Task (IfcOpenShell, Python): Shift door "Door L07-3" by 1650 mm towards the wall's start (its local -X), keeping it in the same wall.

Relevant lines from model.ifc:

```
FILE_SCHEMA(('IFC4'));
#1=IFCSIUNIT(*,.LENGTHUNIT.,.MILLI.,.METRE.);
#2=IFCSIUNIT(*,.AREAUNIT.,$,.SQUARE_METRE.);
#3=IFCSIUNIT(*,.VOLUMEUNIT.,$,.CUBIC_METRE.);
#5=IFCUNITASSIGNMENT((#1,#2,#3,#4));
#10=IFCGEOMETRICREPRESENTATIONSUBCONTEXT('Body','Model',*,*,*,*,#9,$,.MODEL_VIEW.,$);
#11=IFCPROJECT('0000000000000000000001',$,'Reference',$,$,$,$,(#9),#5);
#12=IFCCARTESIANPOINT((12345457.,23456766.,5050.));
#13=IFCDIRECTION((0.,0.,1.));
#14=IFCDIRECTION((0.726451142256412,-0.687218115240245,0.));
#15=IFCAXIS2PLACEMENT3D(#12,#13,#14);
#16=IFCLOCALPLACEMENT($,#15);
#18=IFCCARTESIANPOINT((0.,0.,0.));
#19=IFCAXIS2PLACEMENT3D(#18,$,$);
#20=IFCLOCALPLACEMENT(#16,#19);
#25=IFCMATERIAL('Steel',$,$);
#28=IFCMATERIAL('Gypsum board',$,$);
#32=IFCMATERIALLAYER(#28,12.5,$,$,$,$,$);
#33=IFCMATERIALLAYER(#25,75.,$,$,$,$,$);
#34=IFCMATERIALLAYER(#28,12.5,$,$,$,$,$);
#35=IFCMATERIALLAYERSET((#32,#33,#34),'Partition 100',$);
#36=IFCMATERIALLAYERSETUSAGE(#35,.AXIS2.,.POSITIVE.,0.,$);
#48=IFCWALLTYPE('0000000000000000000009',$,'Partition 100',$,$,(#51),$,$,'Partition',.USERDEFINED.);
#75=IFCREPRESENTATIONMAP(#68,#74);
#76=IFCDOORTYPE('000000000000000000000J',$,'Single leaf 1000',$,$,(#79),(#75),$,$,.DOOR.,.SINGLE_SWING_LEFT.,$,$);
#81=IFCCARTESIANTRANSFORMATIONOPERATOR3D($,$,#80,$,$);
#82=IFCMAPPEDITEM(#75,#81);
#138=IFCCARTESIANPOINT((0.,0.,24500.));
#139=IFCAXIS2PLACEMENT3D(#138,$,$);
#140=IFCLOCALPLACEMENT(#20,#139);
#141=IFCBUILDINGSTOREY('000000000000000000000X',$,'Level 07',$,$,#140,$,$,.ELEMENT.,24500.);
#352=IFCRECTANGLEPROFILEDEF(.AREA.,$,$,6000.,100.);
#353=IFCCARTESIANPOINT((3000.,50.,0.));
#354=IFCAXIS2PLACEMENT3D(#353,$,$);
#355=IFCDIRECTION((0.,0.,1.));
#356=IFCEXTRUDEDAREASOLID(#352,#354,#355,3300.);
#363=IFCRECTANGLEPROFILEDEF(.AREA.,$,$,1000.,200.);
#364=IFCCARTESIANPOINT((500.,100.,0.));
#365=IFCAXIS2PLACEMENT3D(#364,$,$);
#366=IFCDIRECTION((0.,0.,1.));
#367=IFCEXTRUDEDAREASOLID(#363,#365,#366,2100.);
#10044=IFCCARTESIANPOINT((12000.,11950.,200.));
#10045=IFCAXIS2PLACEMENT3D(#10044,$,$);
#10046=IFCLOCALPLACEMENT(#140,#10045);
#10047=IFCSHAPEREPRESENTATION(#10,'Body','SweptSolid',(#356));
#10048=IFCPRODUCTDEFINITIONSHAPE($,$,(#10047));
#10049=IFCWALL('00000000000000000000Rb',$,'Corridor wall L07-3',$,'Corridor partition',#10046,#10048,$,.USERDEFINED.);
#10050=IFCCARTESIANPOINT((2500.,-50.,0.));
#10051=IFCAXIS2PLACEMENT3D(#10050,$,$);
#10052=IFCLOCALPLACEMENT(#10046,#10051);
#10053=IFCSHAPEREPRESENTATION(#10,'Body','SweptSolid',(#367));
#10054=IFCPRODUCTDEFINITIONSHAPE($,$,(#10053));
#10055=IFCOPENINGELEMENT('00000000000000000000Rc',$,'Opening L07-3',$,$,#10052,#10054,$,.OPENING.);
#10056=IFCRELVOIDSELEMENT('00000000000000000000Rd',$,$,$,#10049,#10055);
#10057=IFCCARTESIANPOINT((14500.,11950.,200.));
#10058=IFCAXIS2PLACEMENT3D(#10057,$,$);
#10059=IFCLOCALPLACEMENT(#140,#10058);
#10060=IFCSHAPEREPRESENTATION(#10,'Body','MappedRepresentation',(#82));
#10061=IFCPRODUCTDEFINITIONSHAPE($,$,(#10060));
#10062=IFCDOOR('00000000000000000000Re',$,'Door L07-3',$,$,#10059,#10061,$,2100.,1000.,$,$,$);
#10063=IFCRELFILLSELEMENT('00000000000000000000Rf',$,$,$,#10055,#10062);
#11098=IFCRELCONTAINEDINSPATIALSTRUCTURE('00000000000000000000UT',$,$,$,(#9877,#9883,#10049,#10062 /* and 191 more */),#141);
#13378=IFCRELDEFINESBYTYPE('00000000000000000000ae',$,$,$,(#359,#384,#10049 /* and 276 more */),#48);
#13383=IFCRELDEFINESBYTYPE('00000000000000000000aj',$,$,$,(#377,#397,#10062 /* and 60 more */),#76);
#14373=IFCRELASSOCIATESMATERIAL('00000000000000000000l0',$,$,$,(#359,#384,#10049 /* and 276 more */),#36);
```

```python
import ifcopenshell
import ifcopenshell.api.geometry
import ifcopenshell.util.placement
import ifcopenshell.util.unit

model = ifcopenshell.open("model.ifc")
unit_scale = ifcopenshell.util.unit.calculate_unit_scale(model)

door = model.by_guid("00000000000000000000Re")
opening = door.FillsVoids[0].RelatingOpeningElement
wall = opening.VoidsElements[0].RelatingBuildingElement

wall_matrix = ifcopenshell.util.placement.get_local_placement(wall.ObjectPlacement)
shift = wall_matrix[:3, 0] * -1.65 / unit_scale
before = ifcopenshell.util.placement.get_local_placement(door.ObjectPlacement)[:3, 3].copy()

# The door is not placed relative to its opening, so move both.
for product in (opening, door):
    matrix = ifcopenshell.util.placement.get_local_placement(product.ObjectPlacement)
    matrix[:3, 3] += shift
    ifcopenshell.api.geometry.edit_object_placement(model, product=product, matrix=matrix, is_si=False)

after = ifcopenshell.util.placement.get_local_placement(door.ObjectPlacement)[:3, 3]
print("door moved by", (after - before).round(3) + 0.0)

model.write("model_updated.ifc")
```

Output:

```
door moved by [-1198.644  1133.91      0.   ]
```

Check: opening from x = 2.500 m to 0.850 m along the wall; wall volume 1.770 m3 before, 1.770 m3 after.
